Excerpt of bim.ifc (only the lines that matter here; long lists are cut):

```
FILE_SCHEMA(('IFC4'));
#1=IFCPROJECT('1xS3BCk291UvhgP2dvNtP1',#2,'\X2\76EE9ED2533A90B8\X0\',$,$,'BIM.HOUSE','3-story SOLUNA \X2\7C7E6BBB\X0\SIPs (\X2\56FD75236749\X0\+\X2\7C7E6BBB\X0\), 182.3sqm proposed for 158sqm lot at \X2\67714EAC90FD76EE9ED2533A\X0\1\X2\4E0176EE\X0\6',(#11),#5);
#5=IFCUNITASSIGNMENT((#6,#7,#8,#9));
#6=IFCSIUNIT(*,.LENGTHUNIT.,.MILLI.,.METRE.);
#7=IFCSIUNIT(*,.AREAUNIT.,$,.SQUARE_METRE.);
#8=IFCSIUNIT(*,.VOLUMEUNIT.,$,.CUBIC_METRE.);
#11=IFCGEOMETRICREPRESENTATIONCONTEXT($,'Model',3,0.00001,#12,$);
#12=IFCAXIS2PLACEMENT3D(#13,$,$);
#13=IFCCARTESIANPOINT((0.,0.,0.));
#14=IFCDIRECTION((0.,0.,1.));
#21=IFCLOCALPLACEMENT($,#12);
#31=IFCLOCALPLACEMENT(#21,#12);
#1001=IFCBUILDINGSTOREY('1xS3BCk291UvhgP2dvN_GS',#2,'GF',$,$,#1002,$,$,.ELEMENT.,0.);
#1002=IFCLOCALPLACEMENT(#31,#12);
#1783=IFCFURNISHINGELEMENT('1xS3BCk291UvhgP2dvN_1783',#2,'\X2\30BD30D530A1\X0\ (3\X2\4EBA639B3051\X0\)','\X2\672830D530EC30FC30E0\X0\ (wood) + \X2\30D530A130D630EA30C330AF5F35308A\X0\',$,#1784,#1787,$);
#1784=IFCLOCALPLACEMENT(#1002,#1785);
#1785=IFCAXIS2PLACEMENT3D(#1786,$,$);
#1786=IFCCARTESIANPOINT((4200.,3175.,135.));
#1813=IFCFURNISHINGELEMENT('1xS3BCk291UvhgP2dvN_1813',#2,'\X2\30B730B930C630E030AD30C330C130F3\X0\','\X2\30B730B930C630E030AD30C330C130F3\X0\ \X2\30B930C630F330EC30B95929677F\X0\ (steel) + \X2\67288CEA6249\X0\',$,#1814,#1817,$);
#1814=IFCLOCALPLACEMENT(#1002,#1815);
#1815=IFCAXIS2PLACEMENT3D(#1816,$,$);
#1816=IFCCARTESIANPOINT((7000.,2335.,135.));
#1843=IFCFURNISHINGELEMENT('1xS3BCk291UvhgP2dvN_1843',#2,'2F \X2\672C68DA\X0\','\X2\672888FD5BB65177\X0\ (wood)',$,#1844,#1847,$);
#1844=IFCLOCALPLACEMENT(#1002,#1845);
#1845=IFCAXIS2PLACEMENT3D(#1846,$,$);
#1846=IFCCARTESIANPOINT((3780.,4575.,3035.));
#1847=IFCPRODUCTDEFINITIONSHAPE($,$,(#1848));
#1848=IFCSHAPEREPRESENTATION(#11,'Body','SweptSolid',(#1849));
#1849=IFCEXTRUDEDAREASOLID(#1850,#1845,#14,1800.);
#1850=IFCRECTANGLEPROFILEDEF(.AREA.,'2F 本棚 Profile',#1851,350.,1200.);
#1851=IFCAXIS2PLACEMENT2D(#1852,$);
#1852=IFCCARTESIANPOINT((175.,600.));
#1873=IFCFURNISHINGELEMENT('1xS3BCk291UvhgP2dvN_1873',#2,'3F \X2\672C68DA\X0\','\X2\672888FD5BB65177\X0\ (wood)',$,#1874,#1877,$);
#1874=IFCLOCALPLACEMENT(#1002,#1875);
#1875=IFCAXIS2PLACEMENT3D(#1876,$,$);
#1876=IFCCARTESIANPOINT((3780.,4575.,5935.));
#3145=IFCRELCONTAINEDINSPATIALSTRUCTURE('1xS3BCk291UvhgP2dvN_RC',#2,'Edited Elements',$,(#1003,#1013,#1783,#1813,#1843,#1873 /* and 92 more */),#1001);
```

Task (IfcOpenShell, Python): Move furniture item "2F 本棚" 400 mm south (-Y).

```python
import ifcopenshell
import ifcopenshell.api.geometry
import ifcopenshell.util.placement
import ifcopenshell.util.unit

model = ifcopenshell.open("bim.ifc")
unit_scale = ifcopenshell.util.unit.calculate_unit_scale(model)

item = model.by_guid("1xS3BCk291UvhgP2dvN_1843")
matrix = ifcopenshell.util.placement.get_local_placement(item.ObjectPlacement)
matrix[1, 3] -= 0.4 / unit_scale
ifcopenshell.api.geometry.edit_object_placement(model, product=item, matrix=matrix, is_si=False)

print(ifcopenshell.util.placement.get_local_placement(item.ObjectPlacement).round(3) + 0.0)

model.write("bim_updated.ifc")
```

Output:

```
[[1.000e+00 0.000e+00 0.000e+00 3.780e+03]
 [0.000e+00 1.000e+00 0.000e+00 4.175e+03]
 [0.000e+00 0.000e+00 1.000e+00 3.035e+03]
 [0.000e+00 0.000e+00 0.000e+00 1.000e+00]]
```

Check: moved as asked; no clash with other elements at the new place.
